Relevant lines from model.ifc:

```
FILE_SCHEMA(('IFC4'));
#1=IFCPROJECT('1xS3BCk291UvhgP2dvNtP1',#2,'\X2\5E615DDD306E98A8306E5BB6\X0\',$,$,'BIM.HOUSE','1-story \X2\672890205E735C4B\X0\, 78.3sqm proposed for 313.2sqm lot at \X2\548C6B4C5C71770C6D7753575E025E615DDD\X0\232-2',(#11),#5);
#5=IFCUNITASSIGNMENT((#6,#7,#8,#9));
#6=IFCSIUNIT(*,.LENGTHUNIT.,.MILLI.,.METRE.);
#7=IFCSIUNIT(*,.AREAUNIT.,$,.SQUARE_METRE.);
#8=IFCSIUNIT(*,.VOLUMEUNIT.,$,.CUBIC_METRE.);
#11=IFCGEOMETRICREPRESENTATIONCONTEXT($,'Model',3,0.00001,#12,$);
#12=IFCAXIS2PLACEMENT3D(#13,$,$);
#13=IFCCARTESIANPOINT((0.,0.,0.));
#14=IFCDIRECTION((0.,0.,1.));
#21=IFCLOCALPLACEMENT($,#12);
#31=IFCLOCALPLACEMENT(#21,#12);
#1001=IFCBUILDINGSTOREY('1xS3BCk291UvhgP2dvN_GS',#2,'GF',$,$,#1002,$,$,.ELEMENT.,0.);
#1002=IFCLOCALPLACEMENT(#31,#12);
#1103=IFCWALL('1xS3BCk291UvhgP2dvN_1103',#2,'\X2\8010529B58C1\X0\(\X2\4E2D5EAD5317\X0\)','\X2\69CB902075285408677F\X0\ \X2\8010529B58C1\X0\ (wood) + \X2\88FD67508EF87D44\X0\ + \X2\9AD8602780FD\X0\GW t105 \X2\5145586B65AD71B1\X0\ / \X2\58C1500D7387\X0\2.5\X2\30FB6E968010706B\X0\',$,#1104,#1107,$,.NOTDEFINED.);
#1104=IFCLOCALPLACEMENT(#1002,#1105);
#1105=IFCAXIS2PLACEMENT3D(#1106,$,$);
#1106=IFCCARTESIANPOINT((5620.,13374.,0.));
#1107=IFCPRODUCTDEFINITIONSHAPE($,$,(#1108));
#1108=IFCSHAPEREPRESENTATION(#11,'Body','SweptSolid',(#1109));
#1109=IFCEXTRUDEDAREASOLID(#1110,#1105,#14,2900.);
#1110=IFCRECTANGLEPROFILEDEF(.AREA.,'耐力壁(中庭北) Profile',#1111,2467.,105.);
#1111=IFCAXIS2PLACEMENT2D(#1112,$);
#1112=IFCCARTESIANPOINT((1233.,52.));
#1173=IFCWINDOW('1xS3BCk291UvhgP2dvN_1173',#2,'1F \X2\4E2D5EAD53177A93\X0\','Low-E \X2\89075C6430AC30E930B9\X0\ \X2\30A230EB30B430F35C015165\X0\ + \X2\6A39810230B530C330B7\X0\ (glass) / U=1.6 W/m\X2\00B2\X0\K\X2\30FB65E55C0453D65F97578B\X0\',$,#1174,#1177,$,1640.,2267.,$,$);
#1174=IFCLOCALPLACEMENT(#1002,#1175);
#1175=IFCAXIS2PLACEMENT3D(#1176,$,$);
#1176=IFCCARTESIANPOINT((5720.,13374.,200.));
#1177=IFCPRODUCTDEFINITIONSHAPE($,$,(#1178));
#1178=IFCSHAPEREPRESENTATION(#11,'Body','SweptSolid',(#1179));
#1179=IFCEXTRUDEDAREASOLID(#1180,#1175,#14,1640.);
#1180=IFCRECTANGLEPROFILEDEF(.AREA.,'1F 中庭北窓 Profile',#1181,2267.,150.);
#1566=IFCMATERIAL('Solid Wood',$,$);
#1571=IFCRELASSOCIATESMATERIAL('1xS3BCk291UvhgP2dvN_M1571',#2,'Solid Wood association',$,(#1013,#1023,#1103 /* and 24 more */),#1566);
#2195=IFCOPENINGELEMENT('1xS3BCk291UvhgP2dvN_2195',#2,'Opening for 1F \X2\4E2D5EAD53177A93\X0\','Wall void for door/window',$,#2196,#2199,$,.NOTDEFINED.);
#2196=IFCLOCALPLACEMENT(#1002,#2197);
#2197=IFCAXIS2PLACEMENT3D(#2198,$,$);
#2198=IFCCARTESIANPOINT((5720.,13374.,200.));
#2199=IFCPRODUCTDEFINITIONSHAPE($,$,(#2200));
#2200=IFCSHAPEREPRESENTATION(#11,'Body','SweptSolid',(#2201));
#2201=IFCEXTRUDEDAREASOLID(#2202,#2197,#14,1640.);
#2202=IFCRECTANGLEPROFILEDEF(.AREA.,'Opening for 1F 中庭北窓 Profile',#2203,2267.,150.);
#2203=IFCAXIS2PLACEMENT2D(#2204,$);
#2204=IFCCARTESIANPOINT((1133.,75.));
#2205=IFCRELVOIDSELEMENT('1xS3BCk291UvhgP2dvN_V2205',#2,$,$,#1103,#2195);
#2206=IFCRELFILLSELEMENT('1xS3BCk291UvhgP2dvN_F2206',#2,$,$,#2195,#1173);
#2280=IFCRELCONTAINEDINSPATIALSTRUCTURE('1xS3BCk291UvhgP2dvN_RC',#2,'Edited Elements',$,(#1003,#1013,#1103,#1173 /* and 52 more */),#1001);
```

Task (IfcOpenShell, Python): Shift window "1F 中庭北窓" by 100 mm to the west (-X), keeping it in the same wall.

```python
import ifcopenshell
import ifcopenshell.api.geometry
import ifcopenshell.util.placement
import ifcopenshell.util.unit

model = ifcopenshell.open("model.ifc")
unit_scale = ifcopenshell.util.unit.calculate_unit_scale(model)

window = model.by_guid("1xS3BCk291UvhgP2dvN_1173")
opening = window.FillsVoids[0].RelatingOpeningElement
wall = opening.VoidsElements[0].RelatingBuildingElement

wall_matrix = ifcopenshell.util.placement.get_local_placement(wall.ObjectPlacement)
shift = wall_matrix[:3, 0] * -0.1 / unit_scale
before = ifcopenshell.util.placement.get_local_placement(window.ObjectPlacement)[:3, 3].copy()

# The window is not placed relative to its opening, so move both.
for product in (opening, window):
    matrix = ifcopenshell.util.placement.get_local_placement(product.ObjectPlacement)
    matrix[:3, 3] += shift
    ifcopenshell.api.geometry.edit_object_placement(model, product=product, matrix=matrix, is_si=False)

after = ifcopenshell.util.placement.get_local_placement(window.ObjectPlacement)[:3, 3]
print("window moved by", (after - before).round(3) + 0.0)

model.write("model_updated.ifc")
```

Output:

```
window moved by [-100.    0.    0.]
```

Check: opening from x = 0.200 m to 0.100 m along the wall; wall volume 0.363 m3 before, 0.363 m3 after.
